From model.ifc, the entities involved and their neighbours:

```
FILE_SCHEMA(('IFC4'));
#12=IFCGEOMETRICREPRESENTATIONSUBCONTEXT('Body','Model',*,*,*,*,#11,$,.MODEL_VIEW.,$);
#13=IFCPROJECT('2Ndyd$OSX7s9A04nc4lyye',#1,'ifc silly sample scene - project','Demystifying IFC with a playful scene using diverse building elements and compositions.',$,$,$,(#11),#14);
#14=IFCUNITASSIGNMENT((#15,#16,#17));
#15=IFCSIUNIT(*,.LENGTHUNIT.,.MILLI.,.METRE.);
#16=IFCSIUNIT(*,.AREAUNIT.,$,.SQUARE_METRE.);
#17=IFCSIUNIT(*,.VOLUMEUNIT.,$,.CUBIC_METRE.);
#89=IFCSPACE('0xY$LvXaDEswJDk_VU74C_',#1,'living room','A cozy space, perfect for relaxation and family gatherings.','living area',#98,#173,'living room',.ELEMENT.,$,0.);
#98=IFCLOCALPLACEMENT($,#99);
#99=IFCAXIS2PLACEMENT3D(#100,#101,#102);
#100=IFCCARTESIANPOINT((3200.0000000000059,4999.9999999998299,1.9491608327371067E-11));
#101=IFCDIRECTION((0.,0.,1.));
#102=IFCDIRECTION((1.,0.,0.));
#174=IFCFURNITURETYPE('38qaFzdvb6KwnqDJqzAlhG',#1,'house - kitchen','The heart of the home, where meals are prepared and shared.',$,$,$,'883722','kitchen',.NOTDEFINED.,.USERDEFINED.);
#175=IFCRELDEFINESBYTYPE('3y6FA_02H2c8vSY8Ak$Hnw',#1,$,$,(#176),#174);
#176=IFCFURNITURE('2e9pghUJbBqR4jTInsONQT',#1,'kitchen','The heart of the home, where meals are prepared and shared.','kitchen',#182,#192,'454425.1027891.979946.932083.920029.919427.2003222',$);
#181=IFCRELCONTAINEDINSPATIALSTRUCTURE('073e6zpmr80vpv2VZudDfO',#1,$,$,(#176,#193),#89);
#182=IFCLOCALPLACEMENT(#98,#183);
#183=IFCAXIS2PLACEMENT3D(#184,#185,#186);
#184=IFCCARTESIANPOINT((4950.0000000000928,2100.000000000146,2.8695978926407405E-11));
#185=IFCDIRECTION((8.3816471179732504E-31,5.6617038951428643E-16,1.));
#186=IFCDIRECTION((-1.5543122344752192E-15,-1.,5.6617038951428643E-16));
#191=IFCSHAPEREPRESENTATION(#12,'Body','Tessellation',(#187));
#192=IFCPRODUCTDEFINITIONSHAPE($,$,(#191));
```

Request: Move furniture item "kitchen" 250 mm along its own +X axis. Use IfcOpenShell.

```python
import ifcopenshell
import ifcopenshell.api.geometry
import ifcopenshell.util.placement
import ifcopenshell.util.unit

model = ifcopenshell.open("model.ifc")
unit_scale = ifcopenshell.util.unit.calculate_unit_scale(model)

item = model.by_guid("2e9pghUJbBqR4jTInsONQT")
matrix = ifcopenshell.util.placement.get_local_placement(item.ObjectPlacement)
matrix[:3, 3] += matrix[:3, 0] * 0.25 / unit_scale
ifcopenshell.api.geometry.edit_object_placement(model, product=item, matrix=matrix, is_si=False)

print(ifcopenshell.util.placement.get_local_placement(item.ObjectPlacement).round(3) + 0.0)

model.write("model-out.ifc")
```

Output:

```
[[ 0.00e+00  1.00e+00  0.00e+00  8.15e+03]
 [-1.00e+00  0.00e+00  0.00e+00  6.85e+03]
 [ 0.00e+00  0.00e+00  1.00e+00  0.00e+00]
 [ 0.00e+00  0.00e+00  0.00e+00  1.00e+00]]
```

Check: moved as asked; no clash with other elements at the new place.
